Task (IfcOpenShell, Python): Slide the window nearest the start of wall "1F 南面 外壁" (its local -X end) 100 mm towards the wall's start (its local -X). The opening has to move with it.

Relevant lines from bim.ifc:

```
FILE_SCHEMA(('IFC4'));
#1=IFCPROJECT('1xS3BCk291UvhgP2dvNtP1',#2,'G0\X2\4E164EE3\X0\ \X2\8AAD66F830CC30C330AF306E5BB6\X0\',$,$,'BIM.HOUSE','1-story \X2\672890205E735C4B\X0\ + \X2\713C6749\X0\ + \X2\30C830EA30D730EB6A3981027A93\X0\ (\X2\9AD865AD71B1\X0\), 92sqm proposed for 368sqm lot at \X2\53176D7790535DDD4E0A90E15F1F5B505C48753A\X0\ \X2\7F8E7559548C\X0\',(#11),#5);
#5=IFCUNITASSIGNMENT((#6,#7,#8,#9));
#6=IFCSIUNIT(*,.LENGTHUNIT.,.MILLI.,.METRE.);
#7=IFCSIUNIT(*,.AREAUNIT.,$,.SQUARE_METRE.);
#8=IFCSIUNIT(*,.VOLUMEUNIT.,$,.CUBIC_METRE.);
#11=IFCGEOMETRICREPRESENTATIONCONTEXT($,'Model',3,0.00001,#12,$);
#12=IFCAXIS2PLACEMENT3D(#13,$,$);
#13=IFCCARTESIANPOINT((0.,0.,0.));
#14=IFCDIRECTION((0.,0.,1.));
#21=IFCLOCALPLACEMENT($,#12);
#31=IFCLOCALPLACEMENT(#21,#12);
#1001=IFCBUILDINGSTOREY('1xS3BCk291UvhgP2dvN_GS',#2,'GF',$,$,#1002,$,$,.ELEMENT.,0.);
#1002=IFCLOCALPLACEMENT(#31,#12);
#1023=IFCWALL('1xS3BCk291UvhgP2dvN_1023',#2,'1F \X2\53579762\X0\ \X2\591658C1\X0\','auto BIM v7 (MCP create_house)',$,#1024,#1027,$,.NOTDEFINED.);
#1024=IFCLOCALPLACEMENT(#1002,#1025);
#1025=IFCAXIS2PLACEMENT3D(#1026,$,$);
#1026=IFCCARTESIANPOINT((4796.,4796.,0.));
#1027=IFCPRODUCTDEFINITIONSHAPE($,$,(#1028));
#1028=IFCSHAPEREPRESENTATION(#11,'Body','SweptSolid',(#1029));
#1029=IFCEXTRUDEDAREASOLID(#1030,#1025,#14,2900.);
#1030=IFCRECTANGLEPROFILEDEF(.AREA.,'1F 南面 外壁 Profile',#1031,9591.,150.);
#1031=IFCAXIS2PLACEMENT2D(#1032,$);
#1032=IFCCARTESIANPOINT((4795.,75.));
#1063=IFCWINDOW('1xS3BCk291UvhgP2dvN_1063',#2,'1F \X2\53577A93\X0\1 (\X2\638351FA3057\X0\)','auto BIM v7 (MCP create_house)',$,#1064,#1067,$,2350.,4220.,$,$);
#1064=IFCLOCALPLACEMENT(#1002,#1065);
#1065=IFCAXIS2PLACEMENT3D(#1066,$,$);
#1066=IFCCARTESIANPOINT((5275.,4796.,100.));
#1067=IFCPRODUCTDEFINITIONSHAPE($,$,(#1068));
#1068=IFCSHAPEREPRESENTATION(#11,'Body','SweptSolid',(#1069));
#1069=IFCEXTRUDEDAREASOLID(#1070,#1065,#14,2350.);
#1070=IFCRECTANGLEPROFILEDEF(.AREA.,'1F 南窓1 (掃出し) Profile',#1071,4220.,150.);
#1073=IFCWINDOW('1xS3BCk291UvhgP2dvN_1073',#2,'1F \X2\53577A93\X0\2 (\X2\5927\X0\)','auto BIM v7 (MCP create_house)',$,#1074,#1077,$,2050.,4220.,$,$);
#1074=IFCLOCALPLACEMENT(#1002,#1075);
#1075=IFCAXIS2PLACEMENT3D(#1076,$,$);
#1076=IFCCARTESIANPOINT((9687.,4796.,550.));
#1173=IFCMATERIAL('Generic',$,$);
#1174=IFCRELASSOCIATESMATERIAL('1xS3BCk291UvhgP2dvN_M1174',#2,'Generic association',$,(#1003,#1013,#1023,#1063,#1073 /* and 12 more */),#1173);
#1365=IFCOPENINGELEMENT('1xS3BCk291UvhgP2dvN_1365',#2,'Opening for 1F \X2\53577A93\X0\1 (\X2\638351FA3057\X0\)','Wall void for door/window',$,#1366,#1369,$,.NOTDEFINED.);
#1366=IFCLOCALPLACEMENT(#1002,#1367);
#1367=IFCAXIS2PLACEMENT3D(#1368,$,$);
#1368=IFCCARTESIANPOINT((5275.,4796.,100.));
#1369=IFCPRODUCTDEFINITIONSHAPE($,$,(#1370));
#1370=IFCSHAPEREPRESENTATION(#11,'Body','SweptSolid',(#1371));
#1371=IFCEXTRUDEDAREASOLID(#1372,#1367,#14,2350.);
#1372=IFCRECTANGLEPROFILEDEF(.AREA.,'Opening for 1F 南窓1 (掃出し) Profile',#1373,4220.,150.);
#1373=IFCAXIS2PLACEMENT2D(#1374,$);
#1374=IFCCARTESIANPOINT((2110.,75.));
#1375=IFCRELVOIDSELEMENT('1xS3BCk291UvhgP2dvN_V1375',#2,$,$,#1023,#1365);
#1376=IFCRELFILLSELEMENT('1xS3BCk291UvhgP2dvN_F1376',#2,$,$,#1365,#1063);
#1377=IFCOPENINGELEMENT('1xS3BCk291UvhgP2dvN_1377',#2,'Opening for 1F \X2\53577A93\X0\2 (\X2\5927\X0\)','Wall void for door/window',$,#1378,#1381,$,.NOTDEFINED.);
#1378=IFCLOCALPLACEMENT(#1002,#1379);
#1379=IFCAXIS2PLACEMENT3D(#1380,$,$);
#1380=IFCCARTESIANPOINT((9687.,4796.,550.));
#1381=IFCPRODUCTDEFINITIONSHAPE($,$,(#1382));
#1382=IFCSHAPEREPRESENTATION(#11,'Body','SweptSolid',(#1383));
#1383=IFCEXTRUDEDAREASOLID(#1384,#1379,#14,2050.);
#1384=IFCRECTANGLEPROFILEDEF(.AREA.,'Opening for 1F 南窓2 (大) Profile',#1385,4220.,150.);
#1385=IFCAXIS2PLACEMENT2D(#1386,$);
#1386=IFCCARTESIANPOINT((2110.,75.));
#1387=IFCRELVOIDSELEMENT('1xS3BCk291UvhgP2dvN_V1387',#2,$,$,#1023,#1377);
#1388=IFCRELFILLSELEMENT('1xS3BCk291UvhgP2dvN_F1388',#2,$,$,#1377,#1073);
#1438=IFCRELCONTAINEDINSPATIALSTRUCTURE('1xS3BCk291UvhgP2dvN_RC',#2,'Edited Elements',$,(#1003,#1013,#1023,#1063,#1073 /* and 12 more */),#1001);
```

```python
import ifcopenshell
import ifcopenshell.api.geometry
import ifcopenshell.util.placement
import ifcopenshell.util.unit

model = ifcopenshell.open("bim.ifc")
unit_scale = ifcopenshell.util.unit.calculate_unit_scale(model)

window = model.by_guid("1xS3BCk291UvhgP2dvN_1063")
opening = window.FillsVoids[0].RelatingOpeningElement
wall = opening.VoidsElements[0].RelatingBuildingElement

wall_matrix = ifcopenshell.util.placement.get_local_placement(wall.ObjectPlacement)
shift = wall_matrix[:3, 0] * -0.1 / unit_scale
before = ifcopenshell.util.placement.get_local_placement(window.ObjectPlacement)[:3, 3].copy()

# The window is not placed relative to its opening, so move both.
for product in (opening, window):
    matrix = ifcopenshell.util.placement.get_local_placement(product.ObjectPlacement)
    matrix[:3, 3] += shift
    ifcopenshell.api.geometry.edit_object_placement(model, product=product, matrix=matrix, is_si=False)

after = ifcopenshell.util.placement.get_local_placement(window.ObjectPlacement)[:3, 3]
print("window moved by", (after - before).round(3) + 0.0)

model.write("bim-out.ifc")
```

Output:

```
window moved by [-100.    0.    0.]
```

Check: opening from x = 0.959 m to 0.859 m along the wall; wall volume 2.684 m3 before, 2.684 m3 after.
